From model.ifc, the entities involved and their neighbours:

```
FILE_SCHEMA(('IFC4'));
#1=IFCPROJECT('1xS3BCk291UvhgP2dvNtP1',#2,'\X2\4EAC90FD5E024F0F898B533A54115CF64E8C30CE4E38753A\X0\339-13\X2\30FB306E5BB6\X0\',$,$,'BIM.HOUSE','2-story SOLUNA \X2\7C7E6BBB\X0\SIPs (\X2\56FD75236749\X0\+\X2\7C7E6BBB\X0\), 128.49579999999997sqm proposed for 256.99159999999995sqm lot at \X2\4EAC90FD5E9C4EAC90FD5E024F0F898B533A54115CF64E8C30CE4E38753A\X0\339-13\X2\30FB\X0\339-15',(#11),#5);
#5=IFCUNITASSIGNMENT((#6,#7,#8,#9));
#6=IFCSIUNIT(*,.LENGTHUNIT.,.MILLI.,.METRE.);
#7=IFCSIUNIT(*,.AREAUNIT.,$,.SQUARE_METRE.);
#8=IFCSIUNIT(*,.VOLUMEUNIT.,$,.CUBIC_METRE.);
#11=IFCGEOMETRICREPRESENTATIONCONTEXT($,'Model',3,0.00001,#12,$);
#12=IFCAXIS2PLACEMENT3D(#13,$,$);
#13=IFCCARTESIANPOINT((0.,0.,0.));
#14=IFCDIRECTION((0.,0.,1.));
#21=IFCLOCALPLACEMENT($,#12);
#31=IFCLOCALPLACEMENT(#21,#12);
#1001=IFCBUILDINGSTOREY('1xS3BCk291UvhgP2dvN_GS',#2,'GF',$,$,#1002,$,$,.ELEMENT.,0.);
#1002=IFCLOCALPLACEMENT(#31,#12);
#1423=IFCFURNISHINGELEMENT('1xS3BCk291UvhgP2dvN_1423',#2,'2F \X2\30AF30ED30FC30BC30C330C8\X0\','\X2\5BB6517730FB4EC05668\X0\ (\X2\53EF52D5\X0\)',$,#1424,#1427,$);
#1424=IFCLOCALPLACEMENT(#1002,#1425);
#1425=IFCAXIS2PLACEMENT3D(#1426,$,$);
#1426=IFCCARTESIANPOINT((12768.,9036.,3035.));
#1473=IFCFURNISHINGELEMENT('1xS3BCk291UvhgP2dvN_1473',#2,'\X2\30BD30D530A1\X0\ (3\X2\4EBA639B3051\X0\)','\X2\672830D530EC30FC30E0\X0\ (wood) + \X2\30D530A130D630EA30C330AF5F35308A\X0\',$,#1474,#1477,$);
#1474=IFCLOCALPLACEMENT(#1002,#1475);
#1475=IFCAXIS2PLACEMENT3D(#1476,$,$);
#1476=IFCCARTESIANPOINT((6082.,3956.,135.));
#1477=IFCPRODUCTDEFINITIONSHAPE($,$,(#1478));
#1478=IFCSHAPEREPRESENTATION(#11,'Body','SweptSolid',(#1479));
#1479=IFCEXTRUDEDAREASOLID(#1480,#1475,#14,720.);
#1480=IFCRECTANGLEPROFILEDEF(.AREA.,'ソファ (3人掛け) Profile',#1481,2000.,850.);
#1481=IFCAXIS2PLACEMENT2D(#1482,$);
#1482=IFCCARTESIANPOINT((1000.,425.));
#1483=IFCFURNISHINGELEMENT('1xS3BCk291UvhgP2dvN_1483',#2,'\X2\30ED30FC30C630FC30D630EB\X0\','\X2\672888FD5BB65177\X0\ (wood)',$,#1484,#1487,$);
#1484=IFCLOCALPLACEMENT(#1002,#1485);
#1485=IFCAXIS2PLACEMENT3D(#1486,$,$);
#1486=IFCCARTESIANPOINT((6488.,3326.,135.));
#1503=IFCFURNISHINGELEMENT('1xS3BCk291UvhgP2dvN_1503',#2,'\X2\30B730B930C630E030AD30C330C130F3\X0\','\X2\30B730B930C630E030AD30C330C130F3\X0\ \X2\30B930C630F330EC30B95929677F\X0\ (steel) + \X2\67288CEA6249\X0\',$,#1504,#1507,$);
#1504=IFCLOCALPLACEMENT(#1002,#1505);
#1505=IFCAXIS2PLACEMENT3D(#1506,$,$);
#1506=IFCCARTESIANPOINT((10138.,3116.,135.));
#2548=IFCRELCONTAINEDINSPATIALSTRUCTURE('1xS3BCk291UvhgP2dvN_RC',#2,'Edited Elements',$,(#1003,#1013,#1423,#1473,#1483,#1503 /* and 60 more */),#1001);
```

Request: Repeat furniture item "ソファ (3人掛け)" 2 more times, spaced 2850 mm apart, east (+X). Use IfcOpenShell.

```python
import numpy as np
import ifcopenshell
import ifcopenshell.api.geometry
import ifcopenshell.api.root
import ifcopenshell.util.element
import ifcopenshell.util.placement

model = ifcopenshell.open("model.ifc")


def reuse_history(source, copy):
    """copy_class also copies each property set's owner history, people and application; keep the originals."""
    for rel in copy.IsDefinedBy:
        if rel.is_a("IfcRelDefinesByProperties") and (history := rel.RelatingPropertyDefinition.OwnerHistory):
            rel.RelatingPropertyDefinition.OwnerHistory = source.OwnerHistory
            ifcopenshell.util.element.remove_deep2(model, history)


source = model.by_id(1473)
base = ifcopenshell.util.placement.get_local_placement(source.ObjectPlacement)
step = np.array([1.0, 0.0, 0.0]) * 2850.0

for i in range(1, 3):
    copy = ifcopenshell.api.root.copy_class(model, product=source)
    copy.Representation = ifcopenshell.util.element.copy_deep(
        model, source.Representation, exclude=["IfcGeometricRepresentationContext", "IfcRepresentationMap"]
    )
    reuse_history(source, copy)
    matrix = base.copy()
    matrix[:3, 3] += i * step
    print("added at", matrix[:3, 3].round(3) + 0.0)
    ifcopenshell.api.geometry.edit_object_placement(model, product=copy, matrix=matrix, is_si=False)

model.write("model_updated.ifc")
```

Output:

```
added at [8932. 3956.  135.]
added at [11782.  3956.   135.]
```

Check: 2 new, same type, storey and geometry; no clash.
